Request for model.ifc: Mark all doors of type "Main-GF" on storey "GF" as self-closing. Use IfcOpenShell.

First a look at what the model holds.

```python
import ifcopenshell
import ifcopenshell.util.element

model = ifcopenshell.open("model.ifc")
print(model.schema)
storey = next(s for s in model.by_type("IfcBuildingStorey") if s.Name == "GF")
doors = [e for e in ifcopenshell.util.element.get_decomposition(storey) if e.is_a("IfcDoor")]
seen = {}
for e in doors:
    element_type = ifcopenshell.util.element.get_type(e)
    key = (element_type.Name if element_type != e and element_type else None, ifcopenshell.util.element.get_pset(e, "Pset_DoorCommon", "SelfClosing"))
    seen[key] = seen.get(key, 0) + 1
for (name, value), count in sorted(seen.items(), key=str):
    print(count, "x", name, "|", value)
```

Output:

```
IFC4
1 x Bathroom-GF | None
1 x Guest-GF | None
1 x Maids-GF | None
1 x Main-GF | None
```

```python
import ifcopenshell
import ifcopenshell.api.pset
import ifcopenshell.util.element

model = ifcopenshell.open("model.ifc")

storey = next(s for s in model.by_type("IfcBuildingStorey") if s.Name == "GF")
doors = [e for e in ifcopenshell.util.element.get_decomposition(storey) if e.is_a("IfcDoor")]

count = 0
for e in doors:
    element_type = ifcopenshell.util.element.get_type(e)
    if element_type in (None, e) or element_type.Name != "Main-GF":
        continue
    # add_pset returns the element's existing set when there is one.
    pset = ifcopenshell.api.pset.add_pset(model, product=e, name="Pset_DoorCommon")
    ifcopenshell.api.pset.edit_pset(model, pset=pset, properties={"SelfClosing": True})
    count += 1

print(count, "doors updated")

model.write("model-out.ifc")
```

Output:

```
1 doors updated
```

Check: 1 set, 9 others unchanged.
